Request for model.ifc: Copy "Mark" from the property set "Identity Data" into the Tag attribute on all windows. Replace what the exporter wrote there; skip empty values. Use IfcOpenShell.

First a look at what the model holds.

```python
import ifcopenshell
import ifcopenshell.util.element

model = ifcopenshell.open("model.ifc")
print(model.schema)
windows = model.by_type("IfcWindow")
print(len(windows), "windows")
for e in windows[:8]:
    source = ifcopenshell.util.element.get_pset(e, "Identity Data", "Mark")
    target = e.Tag
    print(e.id(), repr(source), repr(target), sep=" | ")
```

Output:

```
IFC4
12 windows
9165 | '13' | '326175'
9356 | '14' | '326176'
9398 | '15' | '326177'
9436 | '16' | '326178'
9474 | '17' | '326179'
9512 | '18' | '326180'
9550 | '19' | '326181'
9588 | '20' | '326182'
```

```python
import ifcopenshell
import ifcopenshell.util.element

model = ifcopenshell.open("model.ifc")

count = 0
for e in model.by_type("IfcWindow"):
    value = ifcopenshell.util.element.get_pset(e, "Identity Data", "Mark")
    current = e.Tag
    if not value or not value.strip() or current == value:
        continue
    e.Tag = value
    count += 1

print(count, "windows updated")

model.write("model-out.ifc")
```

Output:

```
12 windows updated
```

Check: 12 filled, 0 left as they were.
